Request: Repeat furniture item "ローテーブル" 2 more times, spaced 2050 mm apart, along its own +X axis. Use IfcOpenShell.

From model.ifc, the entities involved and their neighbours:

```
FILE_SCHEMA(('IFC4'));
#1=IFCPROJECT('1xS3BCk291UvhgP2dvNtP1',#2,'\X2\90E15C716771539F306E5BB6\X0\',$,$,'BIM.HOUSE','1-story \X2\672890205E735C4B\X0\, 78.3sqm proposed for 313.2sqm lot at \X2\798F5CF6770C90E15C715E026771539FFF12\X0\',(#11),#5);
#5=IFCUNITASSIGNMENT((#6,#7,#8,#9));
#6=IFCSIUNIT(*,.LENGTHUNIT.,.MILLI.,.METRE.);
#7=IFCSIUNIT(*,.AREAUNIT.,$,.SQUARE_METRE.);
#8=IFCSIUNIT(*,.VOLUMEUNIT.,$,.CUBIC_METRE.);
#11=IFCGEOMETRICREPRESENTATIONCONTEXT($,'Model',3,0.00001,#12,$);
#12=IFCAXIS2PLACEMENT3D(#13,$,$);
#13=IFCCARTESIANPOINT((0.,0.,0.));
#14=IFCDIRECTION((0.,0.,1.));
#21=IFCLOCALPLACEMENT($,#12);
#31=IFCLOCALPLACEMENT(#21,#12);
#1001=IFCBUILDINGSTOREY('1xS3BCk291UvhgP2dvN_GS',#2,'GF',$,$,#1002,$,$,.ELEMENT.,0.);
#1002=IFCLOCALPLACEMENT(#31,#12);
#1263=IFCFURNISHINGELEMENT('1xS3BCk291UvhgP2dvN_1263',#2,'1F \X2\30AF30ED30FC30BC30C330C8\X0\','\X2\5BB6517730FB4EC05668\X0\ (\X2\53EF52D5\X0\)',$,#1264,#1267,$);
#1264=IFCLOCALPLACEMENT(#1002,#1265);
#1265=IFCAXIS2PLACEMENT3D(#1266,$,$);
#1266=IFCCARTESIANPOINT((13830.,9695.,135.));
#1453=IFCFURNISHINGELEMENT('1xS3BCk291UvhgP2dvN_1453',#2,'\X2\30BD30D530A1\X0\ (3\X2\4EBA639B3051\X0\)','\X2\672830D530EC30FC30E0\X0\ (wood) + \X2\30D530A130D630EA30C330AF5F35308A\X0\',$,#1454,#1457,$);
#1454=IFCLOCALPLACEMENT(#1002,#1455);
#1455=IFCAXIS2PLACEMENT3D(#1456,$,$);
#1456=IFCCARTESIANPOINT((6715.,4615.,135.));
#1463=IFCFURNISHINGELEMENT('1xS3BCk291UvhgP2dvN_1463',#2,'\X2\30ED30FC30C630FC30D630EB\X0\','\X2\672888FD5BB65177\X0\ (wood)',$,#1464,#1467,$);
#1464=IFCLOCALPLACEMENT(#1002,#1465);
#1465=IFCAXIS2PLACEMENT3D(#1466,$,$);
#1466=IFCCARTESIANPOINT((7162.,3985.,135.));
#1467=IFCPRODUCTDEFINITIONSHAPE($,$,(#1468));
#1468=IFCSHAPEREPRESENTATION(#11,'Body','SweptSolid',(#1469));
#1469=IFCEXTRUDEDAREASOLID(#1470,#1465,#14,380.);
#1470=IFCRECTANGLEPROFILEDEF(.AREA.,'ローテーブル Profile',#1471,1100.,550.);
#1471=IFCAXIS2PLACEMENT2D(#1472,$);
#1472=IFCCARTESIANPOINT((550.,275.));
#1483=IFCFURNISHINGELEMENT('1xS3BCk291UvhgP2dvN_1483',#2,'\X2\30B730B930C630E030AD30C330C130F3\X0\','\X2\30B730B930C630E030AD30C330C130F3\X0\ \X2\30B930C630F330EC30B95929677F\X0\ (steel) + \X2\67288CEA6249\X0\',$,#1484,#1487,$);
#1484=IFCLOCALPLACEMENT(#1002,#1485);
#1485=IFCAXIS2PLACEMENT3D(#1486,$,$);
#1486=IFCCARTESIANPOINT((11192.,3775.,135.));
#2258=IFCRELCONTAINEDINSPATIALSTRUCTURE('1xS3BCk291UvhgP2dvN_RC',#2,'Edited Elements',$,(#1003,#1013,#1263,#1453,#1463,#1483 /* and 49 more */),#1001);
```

```python
import ifcopenshell
import ifcopenshell.api.geometry
import ifcopenshell.api.root
import ifcopenshell.util.element
import ifcopenshell.util.placement
import ifcopenshell.util.unit

model = ifcopenshell.open("model.ifc")
unit_scale = ifcopenshell.util.unit.calculate_unit_scale(model)


def reuse_history(source, copy):
    """copy_class also copies each property set's owner history, people and application; keep the originals."""
    for rel in copy.IsDefinedBy:
        if rel.is_a("IfcRelDefinesByProperties") and (history := rel.RelatingPropertyDefinition.OwnerHistory):
            rel.RelatingPropertyDefinition.OwnerHistory = source.OwnerHistory
            ifcopenshell.util.element.remove_deep2(model, history)


source = model.by_id(1463)
base = ifcopenshell.util.placement.get_local_placement(source.ObjectPlacement)
step = base[:3, 0] * 2.05 / unit_scale

for i in range(1, 3):
    copy = ifcopenshell.api.root.copy_class(model, product=source)
    copy.Representation = ifcopenshell.util.element.copy_deep(
        model, source.Representation, exclude=["IfcGeometricRepresentationContext", "IfcRepresentationMap"]
    )
    reuse_history(source, copy)
    matrix = base.copy()
    matrix[:3, 3] += i * step
    print("added at", matrix[:3, 3].round(3) + 0.0)
    ifcopenshell.api.geometry.edit_object_placement(model, product=copy, matrix=matrix, is_si=False)

model.write("model-out.ifc")
```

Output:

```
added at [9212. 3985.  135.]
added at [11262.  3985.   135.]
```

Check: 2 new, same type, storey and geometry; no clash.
